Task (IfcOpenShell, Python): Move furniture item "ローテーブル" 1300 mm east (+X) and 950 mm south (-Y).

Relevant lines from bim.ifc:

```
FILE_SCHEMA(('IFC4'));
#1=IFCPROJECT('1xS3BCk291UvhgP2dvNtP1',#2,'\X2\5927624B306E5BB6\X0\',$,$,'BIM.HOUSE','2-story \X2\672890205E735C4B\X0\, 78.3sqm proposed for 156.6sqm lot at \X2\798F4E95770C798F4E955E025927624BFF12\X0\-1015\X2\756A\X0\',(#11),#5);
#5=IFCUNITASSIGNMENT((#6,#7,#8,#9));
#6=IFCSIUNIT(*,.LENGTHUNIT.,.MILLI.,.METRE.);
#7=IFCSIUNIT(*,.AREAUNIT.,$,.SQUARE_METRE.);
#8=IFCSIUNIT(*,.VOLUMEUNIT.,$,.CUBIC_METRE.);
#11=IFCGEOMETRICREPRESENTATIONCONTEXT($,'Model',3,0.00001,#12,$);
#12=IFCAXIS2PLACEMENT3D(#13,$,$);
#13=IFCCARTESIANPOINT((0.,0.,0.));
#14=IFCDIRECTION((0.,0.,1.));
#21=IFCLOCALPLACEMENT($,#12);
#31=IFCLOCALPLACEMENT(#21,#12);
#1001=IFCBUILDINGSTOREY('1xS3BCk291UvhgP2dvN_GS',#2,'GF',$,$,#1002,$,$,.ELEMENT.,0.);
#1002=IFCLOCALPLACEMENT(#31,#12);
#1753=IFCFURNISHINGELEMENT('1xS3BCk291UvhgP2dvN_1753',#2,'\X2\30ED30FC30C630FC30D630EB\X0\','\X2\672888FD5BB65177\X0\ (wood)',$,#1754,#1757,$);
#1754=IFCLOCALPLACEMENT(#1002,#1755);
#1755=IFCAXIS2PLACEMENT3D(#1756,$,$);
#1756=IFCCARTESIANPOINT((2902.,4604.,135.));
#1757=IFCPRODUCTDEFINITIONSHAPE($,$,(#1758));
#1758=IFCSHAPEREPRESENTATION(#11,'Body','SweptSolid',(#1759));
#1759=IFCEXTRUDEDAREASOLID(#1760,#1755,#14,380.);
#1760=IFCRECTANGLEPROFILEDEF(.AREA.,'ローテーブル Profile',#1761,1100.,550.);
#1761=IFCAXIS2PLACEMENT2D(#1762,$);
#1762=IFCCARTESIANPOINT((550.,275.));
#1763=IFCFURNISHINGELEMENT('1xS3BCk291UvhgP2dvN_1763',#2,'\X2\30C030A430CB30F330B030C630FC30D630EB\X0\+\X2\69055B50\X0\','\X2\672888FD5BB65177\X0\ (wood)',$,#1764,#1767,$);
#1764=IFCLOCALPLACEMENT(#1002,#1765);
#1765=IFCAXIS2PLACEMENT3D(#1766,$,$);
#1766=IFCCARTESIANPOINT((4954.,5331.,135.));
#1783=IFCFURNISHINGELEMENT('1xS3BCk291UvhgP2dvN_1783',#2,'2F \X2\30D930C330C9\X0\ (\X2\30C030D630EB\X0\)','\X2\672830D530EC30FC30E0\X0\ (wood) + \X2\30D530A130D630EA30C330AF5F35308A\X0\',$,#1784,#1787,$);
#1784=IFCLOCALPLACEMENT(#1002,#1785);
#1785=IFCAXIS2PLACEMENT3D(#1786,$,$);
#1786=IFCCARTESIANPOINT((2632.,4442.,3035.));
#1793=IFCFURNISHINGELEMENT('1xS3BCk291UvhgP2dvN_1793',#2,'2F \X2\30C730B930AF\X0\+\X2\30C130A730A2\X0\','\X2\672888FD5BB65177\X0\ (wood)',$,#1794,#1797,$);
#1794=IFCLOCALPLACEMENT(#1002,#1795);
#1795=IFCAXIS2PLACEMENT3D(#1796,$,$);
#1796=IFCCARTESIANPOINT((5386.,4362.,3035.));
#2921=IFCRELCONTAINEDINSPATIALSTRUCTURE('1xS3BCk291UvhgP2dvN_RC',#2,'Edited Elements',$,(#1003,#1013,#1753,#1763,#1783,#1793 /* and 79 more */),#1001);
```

```python
import ifcopenshell
import ifcopenshell.api.geometry
import ifcopenshell.util.placement

model = ifcopenshell.open("bim.ifc")

item = model.by_guid("1xS3BCk291UvhgP2dvN_1753")
matrix = ifcopenshell.util.placement.get_local_placement(item.ObjectPlacement)
matrix[0, 3] += 1300.0
matrix[1, 3] -= 950.0
ifcopenshell.api.geometry.edit_object_placement(model, product=item, matrix=matrix, is_si=False)

print(ifcopenshell.util.placement.get_local_placement(item.ObjectPlacement).round(3) + 0.0)

model.write("bim-out.ifc")
```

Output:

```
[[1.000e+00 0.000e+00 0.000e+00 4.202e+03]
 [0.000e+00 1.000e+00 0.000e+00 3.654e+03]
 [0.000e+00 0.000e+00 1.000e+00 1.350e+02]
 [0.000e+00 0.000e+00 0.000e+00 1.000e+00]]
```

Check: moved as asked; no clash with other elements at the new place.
